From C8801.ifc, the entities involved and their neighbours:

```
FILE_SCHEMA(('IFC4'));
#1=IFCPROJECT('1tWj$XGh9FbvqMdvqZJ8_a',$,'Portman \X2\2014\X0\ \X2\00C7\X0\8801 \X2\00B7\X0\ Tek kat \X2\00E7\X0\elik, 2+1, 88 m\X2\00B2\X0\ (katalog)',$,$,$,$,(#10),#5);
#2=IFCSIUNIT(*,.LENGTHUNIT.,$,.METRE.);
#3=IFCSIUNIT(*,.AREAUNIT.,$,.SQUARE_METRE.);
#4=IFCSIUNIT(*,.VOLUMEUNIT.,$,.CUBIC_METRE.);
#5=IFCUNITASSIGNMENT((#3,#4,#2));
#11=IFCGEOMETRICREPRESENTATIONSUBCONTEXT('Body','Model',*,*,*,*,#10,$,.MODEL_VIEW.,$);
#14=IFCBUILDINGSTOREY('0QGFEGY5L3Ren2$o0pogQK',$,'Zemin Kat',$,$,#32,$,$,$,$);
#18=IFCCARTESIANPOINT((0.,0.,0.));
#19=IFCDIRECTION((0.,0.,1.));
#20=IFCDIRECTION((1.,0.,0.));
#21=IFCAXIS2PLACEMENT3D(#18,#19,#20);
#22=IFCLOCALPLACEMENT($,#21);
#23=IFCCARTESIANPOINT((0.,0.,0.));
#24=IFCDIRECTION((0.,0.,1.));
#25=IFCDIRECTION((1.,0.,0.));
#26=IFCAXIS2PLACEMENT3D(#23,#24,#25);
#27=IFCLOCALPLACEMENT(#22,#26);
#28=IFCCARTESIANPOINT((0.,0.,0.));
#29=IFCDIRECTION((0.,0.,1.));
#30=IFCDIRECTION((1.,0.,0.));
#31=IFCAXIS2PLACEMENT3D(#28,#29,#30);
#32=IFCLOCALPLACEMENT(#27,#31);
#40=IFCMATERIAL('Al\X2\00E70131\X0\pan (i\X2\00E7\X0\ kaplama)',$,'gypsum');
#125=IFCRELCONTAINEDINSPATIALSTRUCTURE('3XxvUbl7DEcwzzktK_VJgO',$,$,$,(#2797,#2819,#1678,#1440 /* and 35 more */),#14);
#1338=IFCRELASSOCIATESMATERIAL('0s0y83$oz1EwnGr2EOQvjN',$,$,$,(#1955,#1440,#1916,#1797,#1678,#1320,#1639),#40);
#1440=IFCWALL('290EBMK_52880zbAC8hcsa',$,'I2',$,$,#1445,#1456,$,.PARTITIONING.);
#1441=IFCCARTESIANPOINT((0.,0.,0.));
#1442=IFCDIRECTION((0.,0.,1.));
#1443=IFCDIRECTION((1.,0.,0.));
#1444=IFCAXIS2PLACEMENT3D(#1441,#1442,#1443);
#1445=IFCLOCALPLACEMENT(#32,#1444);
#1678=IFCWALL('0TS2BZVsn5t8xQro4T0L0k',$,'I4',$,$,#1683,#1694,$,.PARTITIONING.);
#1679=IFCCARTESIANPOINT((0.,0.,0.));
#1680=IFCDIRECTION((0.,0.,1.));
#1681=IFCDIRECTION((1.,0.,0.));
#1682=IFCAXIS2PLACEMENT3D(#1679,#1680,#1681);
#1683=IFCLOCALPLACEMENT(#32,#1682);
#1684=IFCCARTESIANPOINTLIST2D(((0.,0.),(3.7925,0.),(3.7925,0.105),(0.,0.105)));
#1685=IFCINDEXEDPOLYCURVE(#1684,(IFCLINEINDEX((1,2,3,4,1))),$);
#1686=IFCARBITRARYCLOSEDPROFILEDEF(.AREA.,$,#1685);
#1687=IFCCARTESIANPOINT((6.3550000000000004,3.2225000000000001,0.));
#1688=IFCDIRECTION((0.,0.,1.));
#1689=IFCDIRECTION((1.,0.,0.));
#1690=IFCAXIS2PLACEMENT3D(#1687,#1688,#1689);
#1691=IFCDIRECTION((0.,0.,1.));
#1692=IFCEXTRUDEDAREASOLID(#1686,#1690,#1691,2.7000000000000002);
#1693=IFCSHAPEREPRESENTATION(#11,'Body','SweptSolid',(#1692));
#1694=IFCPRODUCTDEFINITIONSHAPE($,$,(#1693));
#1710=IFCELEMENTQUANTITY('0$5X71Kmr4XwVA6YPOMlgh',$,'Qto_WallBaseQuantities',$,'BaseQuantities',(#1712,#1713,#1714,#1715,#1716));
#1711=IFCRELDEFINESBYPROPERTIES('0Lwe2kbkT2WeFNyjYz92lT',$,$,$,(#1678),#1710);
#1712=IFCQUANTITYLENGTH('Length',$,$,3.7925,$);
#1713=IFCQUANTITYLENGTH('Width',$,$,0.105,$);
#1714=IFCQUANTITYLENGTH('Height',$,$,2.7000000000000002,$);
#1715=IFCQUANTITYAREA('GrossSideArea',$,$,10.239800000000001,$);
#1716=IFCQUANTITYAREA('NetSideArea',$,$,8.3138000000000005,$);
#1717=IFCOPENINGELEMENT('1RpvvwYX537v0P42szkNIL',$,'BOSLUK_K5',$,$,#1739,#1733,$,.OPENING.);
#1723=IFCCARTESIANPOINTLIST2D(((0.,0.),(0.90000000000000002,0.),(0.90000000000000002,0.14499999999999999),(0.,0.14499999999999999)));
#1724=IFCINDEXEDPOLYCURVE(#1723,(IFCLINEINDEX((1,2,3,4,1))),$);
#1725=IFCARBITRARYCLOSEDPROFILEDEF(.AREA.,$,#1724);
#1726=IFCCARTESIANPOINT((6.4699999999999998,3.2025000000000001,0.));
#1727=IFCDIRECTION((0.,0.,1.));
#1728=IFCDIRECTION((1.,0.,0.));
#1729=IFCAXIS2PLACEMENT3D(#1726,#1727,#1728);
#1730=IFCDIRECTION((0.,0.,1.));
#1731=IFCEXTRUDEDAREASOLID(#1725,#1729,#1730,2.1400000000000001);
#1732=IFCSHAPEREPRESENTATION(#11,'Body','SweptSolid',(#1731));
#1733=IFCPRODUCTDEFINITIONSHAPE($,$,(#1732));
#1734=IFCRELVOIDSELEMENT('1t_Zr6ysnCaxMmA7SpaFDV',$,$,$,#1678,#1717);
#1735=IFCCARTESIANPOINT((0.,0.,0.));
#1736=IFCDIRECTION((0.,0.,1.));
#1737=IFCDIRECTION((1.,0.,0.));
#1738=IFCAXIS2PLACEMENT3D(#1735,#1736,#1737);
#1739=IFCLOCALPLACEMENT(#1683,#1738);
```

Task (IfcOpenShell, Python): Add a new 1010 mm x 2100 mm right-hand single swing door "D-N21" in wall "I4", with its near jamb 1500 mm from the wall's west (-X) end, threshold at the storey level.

```python
import numpy as np
import ifcopenshell
import ifcopenshell.api.feature
import ifcopenshell.api.geometry
import ifcopenshell.api.pset
import ifcopenshell.api.root
import ifcopenshell.api.spatial
import ifcopenshell.geom
import ifcopenshell.util.element
import ifcopenshell.util.placement
import ifcopenshell.util.representation
import ifcopenshell.util.shape
import ifcopenshell.util.unit

model = ifcopenshell.open("C8801.ifc")
unit_scale = ifcopenshell.util.unit.calculate_unit_scale(model)
area_scale = ifcopenshell.util.unit.calculate_unit_scale(model, "AREAUNIT")
settings = ifcopenshell.geom.settings()


def volume(element):
    """Net volume in cubic metres, openings subtracted."""
    shape = ifcopenshell.geom.create_shape(settings, element)
    return ifcopenshell.util.shape.get_volume(shape.geometry)


wall = model.by_guid("0TS2BZVsn5t8xQro4T0L0k")
storey = ifcopenshell.util.element.get_container(wall, ifc_class="IfcBuildingStorey")
context = ifcopenshell.util.representation.get_context(model, "Model", "Body", "MODEL_VIEW")
before = volume(wall)

width, height, from_end, sill = 1.01, 2.1, 1.5, 0.0  # metres

# The wall runs along its own X axis, and the end named is its -X end.
wall_shape = ifcopenshell.geom.create_shape(settings, wall)
x, y, z = ifcopenshell.util.shape.get_vertices(wall_shape.geometry).T
start = x.min() + from_end
face, thickness = float(y.min()), float(y.max() - y.min())
wall_matrix = ifcopenshell.util.placement.get_local_placement(wall.ObjectPlacement)
level = ifcopenshell.util.placement.get_local_placement(storey.ObjectPlacement)[2, 3]


def in_wall(x, y):
    """Placement at x, y metres in the wall's axes, at sill height."""
    matrix = wall_matrix.copy()
    matrix[:, 3] = wall_matrix @ np.array([x / unit_scale, y / unit_scale, 0.0, 1.0])
    matrix[2, 3] = level + sill / unit_scale
    return matrix


# Opening: a box that overshoots both wall faces by 50 mm.
opening = ifcopenshell.api.root.create_entity(model, ifc_class="IfcOpeningElement", predefined_type="OPENING")
box = ifcopenshell.api.geometry.add_wall_representation(
    model, context=context, length=width, height=height, thickness=thickness + 0.1
)
ifcopenshell.api.geometry.assign_representation(model, product=opening, representation=box)
ifcopenshell.api.geometry.edit_object_placement(model, product=opening, matrix=in_wall(start, face - 0.05), is_si=False)
ifcopenshell.api.feature.add_feature(model, feature=opening, element=wall)

door = ifcopenshell.api.root.create_entity(model, ifc_class="IfcDoor", name="D-N21", predefined_type="DOOR")
door.OverallWidth, door.OverallHeight = width / unit_scale, height / unit_scale
door.OperationType = "SINGLE_SWING_RIGHT"
body = ifcopenshell.api.geometry.add_door_representation(
    model,
    context=context,
    overall_width=door.OverallWidth,
    overall_height=door.OverallHeight,
    operation_type="SINGLE_SWING_RIGHT",
    lining_properties={"LiningDepth": thickness / unit_scale, "ThresholdDepth": thickness / unit_scale},
)
ifcopenshell.api.geometry.assign_representation(model, product=door, representation=body)
ifcopenshell.api.spatial.assign_container(model, products=[door], relating_structure=storey)
ifcopenshell.api.feature.add_filling(model, opening=opening, element=door)

# The lining spans the wall, so the door starts at the wall face.
ifcopenshell.api.geometry.edit_object_placement(model, product=door, matrix=in_wall(start, face), is_si=False)

after = volume(wall)

# Update the wall's stored quantities.
qto = model.by_id(ifcopenshell.util.element.get_pset(wall, "Qto_WallBaseQuantities", should_inherit=False)["id"])
ifcopenshell.api.pset.edit_qto(model, qto=qto, properties={"NetSideArea": after / thickness / area_scale})

print(f"wall volume {before:.3f} -> {after:.3f} m3")

model.write("C8801_rev.ifc")
```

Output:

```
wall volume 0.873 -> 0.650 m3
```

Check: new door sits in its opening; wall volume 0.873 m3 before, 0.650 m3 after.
